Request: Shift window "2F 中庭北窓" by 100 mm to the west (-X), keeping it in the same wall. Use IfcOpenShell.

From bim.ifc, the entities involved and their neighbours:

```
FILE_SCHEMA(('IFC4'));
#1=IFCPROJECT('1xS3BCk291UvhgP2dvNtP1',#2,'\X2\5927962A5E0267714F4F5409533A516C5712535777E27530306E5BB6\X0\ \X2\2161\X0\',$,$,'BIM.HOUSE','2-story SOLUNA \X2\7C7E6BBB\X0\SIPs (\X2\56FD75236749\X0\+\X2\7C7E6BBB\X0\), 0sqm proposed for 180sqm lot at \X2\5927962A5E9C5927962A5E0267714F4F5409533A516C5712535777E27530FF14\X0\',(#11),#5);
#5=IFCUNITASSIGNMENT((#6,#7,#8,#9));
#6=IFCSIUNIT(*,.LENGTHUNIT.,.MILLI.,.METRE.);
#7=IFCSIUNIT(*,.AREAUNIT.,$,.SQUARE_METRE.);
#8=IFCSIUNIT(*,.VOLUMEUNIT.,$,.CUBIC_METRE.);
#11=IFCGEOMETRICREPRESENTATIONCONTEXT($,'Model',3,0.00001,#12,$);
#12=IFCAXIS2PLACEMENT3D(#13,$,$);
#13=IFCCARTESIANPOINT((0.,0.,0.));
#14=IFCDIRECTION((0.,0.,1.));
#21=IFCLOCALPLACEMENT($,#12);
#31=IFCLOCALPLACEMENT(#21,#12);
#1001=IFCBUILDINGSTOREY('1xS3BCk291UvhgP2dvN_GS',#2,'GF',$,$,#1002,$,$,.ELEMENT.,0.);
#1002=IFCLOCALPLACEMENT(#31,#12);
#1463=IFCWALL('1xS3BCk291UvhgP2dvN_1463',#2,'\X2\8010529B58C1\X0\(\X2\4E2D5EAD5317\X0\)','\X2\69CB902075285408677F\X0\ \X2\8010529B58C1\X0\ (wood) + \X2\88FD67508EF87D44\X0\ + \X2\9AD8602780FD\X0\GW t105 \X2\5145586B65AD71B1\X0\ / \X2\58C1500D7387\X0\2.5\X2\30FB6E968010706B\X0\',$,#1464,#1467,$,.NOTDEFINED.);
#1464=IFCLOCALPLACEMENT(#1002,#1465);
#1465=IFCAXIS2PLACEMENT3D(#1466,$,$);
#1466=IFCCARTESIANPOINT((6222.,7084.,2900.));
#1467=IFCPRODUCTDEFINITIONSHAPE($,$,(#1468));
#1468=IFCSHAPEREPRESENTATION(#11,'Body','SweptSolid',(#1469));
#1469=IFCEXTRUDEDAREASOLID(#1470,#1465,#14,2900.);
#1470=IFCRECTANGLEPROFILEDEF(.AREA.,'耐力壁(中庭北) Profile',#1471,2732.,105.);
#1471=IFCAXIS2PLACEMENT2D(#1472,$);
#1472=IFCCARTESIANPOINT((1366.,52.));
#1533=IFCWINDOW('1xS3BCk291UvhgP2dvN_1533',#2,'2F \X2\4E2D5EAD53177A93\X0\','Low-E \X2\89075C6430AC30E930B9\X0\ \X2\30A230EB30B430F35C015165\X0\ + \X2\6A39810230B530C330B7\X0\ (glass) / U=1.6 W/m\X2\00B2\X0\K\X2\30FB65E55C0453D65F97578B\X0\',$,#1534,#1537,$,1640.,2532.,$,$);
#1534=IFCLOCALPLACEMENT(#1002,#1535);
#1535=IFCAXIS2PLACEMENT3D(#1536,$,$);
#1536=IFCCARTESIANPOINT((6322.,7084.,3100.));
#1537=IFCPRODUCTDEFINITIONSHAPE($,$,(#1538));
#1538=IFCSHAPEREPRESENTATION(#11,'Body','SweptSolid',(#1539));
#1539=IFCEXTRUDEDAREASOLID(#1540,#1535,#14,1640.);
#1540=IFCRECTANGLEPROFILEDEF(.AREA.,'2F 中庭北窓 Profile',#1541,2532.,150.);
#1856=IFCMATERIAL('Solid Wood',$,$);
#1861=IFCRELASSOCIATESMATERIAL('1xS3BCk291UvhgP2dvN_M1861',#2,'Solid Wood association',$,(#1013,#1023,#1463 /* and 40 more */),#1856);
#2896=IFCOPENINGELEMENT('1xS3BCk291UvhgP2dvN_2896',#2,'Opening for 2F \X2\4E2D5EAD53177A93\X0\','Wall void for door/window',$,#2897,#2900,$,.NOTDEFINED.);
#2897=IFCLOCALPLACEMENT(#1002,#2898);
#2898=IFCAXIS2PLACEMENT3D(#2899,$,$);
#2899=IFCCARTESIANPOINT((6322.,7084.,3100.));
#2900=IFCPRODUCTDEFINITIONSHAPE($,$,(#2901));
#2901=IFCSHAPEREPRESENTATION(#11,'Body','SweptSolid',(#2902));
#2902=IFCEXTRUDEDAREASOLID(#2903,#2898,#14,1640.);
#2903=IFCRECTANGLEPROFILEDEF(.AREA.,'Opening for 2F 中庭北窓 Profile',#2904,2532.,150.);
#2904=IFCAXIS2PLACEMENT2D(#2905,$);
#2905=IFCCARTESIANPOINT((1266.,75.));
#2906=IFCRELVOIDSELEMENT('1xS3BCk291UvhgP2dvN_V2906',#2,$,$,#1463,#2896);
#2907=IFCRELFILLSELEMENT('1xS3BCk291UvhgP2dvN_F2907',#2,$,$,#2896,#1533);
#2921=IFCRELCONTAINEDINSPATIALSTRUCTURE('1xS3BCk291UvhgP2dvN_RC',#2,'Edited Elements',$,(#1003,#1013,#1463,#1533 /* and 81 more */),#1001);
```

```python
import ifcopenshell
import ifcopenshell.api.geometry
import ifcopenshell.util.placement
import ifcopenshell.util.unit

model = ifcopenshell.open("bim.ifc")
unit_scale = ifcopenshell.util.unit.calculate_unit_scale(model)

window = model.by_guid("1xS3BCk291UvhgP2dvN_1533")
opening = window.FillsVoids[0].RelatingOpeningElement
wall = opening.VoidsElements[0].RelatingBuildingElement

wall_matrix = ifcopenshell.util.placement.get_local_placement(wall.ObjectPlacement)
shift = wall_matrix[:3, 0] * -0.1 / unit_scale
before = ifcopenshell.util.placement.get_local_placement(window.ObjectPlacement)[:3, 3].copy()

# The window is not placed relative to its opening, so move both.
for product in (opening, window):
    matrix = ifcopenshell.util.placement.get_local_placement(product.ObjectPlacement)
    matrix[:3, 3] += shift
    ifcopenshell.api.geometry.edit_object_placement(model, product=product, matrix=matrix, is_si=False)

after = ifcopenshell.util.placement.get_local_placement(window.ObjectPlacement)[:3, 3]
print("window moved by", (after - before).round(3) + 0.0)

model.write("bim_v2.ifc")
```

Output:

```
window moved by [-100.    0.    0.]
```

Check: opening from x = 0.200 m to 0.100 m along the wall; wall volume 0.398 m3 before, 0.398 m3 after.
